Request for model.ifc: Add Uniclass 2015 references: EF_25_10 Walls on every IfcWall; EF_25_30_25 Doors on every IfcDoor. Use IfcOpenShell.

First a look at what the model holds.

```python
import ifcopenshell

model = ifcopenshell.open("model.ifc")
print(model.schema)
print("classifications:", [c.Name for c in model.by_type("IfcClassification")])
for ifc_class in ("IfcDoor", "IfcRoof", "IfcStair", "IfcWall", "IfcWindow"):
    print(ifc_class, len(model.by_type(ifc_class)))
```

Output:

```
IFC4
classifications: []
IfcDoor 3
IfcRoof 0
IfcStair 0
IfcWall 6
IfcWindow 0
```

```python
import ifcopenshell
import ifcopenshell.api.classification

model = ifcopenshell.open("model.ifc")

system = ifcopenshell.api.classification.add_classification(model, classification="Uniclass 2015")

codes = {
    "IfcWall": ("EF_25_10", "Walls"),
    "IfcDoor": ("EF_25_30_25", "Doors"),
}
for ifc_class, (code, name) in codes.items():
    products = model.by_type(ifc_class)
    ifcopenshell.api.classification.add_reference(
        model, products=products, classification=system, identification=code, name=name
    )
    print(code, len(products))

model.write("model_v2.ifc")
```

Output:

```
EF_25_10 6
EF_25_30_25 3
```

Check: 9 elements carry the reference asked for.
